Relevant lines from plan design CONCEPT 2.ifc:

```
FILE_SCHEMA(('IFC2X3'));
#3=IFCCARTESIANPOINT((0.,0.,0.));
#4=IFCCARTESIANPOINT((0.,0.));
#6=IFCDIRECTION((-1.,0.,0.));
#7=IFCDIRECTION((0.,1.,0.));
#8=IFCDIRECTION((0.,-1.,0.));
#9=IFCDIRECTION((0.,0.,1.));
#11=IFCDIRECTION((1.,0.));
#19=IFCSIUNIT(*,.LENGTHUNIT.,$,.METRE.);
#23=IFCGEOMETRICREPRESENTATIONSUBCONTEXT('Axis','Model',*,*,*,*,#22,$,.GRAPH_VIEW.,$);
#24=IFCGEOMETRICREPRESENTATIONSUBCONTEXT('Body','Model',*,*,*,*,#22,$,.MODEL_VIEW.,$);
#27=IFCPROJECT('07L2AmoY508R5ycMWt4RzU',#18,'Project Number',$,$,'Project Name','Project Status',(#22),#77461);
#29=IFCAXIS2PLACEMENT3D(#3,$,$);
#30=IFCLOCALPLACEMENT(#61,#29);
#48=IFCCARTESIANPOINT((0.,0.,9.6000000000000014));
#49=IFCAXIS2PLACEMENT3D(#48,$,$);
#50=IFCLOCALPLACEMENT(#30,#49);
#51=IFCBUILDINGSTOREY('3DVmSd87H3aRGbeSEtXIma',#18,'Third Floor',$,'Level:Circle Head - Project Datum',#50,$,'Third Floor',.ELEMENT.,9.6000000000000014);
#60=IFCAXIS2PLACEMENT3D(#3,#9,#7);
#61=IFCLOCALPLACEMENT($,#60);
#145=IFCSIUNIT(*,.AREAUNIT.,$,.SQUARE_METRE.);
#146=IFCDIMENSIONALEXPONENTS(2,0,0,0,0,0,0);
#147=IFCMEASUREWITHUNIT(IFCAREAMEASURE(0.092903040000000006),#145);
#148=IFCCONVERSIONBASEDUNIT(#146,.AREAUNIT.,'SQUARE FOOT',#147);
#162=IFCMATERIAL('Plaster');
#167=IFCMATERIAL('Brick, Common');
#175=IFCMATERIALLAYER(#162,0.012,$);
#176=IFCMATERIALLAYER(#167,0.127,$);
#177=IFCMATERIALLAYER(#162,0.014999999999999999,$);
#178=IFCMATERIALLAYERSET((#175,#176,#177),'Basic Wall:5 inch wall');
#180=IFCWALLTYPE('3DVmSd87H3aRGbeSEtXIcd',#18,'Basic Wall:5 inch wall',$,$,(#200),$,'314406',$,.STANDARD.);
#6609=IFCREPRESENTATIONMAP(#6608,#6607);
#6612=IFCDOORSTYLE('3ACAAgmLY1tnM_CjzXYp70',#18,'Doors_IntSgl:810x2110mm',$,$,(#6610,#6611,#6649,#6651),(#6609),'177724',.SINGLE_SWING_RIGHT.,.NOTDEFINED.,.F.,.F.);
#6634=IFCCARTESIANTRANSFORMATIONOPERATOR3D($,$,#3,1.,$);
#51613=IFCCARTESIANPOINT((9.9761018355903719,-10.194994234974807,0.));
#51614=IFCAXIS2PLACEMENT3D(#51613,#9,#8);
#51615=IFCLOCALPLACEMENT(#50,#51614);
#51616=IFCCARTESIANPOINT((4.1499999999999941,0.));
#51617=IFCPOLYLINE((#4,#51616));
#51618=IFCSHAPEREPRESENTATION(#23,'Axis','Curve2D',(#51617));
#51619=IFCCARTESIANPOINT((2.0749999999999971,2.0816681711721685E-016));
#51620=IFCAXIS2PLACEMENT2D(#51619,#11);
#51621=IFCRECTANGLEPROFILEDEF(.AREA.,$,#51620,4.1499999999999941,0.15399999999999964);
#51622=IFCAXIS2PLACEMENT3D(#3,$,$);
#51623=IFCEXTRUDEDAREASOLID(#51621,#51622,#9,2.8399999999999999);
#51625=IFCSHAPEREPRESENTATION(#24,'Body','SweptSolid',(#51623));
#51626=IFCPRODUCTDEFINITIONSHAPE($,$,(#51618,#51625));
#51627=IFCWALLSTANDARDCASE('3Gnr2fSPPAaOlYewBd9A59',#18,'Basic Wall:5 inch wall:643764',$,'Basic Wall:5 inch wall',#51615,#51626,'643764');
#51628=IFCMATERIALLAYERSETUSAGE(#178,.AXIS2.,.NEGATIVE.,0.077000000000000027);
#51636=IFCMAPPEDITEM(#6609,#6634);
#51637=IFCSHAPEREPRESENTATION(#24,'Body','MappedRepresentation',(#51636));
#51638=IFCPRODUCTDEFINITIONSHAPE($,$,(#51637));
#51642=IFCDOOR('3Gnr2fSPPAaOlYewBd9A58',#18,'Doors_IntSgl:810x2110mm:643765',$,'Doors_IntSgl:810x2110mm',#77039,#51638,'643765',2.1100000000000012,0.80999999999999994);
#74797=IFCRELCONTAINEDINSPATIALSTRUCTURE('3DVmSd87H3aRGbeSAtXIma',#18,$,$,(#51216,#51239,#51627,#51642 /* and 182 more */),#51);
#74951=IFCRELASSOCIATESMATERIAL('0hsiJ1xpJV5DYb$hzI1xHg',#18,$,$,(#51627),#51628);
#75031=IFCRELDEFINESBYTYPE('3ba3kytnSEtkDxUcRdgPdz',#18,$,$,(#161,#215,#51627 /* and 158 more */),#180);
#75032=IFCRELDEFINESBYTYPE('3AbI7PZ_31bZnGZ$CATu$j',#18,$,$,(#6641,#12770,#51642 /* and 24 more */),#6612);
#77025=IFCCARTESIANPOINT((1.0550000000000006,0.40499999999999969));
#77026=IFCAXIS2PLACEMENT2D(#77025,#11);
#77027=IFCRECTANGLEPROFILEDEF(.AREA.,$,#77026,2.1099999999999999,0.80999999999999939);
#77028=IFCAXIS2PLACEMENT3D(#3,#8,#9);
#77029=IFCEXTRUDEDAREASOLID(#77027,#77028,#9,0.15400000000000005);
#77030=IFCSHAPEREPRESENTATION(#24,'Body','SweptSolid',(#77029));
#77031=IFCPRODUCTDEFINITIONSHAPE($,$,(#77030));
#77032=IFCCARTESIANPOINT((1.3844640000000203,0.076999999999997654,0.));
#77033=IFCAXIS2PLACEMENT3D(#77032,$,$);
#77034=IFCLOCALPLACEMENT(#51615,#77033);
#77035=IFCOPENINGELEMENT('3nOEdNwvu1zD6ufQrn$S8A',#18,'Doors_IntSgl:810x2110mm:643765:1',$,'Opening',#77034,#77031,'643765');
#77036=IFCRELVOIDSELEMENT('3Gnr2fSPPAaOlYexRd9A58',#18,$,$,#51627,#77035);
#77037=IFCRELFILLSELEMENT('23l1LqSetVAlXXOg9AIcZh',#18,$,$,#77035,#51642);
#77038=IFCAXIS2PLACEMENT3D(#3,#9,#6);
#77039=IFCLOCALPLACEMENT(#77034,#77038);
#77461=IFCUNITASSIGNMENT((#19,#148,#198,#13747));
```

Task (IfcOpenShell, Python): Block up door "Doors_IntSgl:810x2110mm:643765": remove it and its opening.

```python
import ifcopenshell
import ifcopenshell.api.feature
import ifcopenshell.api.root
import ifcopenshell.geom
import ifcopenshell.util.shape

model = ifcopenshell.open("plan design CONCEPT 2.ifc")
settings = ifcopenshell.geom.settings()


def volume(element):
    """Net volume in cubic metres, openings subtracted."""
    shape = ifcopenshell.geom.create_shape(settings, element)
    return ifcopenshell.util.shape.get_volume(shape.geometry)


door = model.by_guid("3Gnr2fSPPAaOlYewBd9A58")
opening = door.FillsVoids[0].RelatingOpeningElement
wall = opening.VoidsElements[0].RelatingBuildingElement
before = volume(wall)

ifcopenshell.api.root.remove_product(model, product=door)
ifcopenshell.api.feature.remove_feature(model, feature=opening)

after = volume(wall)

print(f"wall volume {before:.3f} -> {after:.3f} m3")

model.write("plan design CONCEPT 2_updated.ifc")
```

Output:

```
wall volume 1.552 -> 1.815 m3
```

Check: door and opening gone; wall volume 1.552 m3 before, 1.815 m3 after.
